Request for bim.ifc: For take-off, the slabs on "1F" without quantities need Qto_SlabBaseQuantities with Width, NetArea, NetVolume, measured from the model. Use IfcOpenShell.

First a look at what the model holds.

```python
import ifcopenshell
import ifcopenshell.util.element
import ifcopenshell.util.unit

model = ifcopenshell.open("bim.ifc")
print(model.schema)
for unit_type in ("LENGTHUNIT", "AREAUNIT", "VOLUMEUNIT"):
    print(unit_type, ifcopenshell.util.unit.calculate_unit_scale(model, unit_type))
storey = next(s for s in model.by_type("IfcBuildingStorey") if s.Name == "1F")
slabs = [e for e in ifcopenshell.util.element.get_decomposition(storey) if e.is_a("IfcSlab")]
for e in sorted(slabs, key=lambda e: e.id()):
    print(e.id(), e.is_a(), e.Name, list(ifcopenshell.util.element.get_psets(e, qtos_only=True)), sep=" | ")
```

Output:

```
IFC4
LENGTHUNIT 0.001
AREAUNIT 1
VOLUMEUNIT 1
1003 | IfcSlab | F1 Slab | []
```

```python
import ifcopenshell
import ifcopenshell.api.pset
import ifcopenshell.geom
import ifcopenshell.util.element
import ifcopenshell.util.shape
import ifcopenshell.util.unit

model = ifcopenshell.open("bim.ifc")
unit_scale = ifcopenshell.util.unit.calculate_unit_scale(model)
area_scale = ifcopenshell.util.unit.calculate_unit_scale(model, "AREAUNIT")
volume_scale = ifcopenshell.util.unit.calculate_unit_scale(model, "VOLUMEUNIT")
settings = ifcopenshell.geom.settings()

storey = next(s for s in model.by_type("IfcBuildingStorey") if s.Name == "1F")
slabs = [e for e in ifcopenshell.util.element.get_decomposition(storey) if e.is_a("IfcSlab")]

for e in sorted(slabs, key=lambda e: e.id()):
    if ifcopenshell.util.element.get_psets(e, qtos_only=True, should_inherit=False):
        continue
    # Geometry comes back in metres, in the element's own axes.
    shape = ifcopenshell.geom.create_shape(settings, e)
    values = {
        "Width": ifcopenshell.util.shape.get_z(shape.geometry) / unit_scale,
        "NetArea": ifcopenshell.util.shape.get_footprint_area(shape.geometry) / area_scale,
        "NetVolume": ifcopenshell.util.shape.get_volume(shape.geometry) / volume_scale,
    }
    qto = ifcopenshell.api.pset.add_qto(model, product=e, name="Qto_SlabBaseQuantities")
    ifcopenshell.api.pset.edit_qto(model, qto=qto, properties=values)
    print(e.id(), {k: round(v, 3) for k, v in values.items()})

model.write("bim_v2.ifc")
```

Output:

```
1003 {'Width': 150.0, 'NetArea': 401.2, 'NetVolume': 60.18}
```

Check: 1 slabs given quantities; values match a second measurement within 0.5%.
